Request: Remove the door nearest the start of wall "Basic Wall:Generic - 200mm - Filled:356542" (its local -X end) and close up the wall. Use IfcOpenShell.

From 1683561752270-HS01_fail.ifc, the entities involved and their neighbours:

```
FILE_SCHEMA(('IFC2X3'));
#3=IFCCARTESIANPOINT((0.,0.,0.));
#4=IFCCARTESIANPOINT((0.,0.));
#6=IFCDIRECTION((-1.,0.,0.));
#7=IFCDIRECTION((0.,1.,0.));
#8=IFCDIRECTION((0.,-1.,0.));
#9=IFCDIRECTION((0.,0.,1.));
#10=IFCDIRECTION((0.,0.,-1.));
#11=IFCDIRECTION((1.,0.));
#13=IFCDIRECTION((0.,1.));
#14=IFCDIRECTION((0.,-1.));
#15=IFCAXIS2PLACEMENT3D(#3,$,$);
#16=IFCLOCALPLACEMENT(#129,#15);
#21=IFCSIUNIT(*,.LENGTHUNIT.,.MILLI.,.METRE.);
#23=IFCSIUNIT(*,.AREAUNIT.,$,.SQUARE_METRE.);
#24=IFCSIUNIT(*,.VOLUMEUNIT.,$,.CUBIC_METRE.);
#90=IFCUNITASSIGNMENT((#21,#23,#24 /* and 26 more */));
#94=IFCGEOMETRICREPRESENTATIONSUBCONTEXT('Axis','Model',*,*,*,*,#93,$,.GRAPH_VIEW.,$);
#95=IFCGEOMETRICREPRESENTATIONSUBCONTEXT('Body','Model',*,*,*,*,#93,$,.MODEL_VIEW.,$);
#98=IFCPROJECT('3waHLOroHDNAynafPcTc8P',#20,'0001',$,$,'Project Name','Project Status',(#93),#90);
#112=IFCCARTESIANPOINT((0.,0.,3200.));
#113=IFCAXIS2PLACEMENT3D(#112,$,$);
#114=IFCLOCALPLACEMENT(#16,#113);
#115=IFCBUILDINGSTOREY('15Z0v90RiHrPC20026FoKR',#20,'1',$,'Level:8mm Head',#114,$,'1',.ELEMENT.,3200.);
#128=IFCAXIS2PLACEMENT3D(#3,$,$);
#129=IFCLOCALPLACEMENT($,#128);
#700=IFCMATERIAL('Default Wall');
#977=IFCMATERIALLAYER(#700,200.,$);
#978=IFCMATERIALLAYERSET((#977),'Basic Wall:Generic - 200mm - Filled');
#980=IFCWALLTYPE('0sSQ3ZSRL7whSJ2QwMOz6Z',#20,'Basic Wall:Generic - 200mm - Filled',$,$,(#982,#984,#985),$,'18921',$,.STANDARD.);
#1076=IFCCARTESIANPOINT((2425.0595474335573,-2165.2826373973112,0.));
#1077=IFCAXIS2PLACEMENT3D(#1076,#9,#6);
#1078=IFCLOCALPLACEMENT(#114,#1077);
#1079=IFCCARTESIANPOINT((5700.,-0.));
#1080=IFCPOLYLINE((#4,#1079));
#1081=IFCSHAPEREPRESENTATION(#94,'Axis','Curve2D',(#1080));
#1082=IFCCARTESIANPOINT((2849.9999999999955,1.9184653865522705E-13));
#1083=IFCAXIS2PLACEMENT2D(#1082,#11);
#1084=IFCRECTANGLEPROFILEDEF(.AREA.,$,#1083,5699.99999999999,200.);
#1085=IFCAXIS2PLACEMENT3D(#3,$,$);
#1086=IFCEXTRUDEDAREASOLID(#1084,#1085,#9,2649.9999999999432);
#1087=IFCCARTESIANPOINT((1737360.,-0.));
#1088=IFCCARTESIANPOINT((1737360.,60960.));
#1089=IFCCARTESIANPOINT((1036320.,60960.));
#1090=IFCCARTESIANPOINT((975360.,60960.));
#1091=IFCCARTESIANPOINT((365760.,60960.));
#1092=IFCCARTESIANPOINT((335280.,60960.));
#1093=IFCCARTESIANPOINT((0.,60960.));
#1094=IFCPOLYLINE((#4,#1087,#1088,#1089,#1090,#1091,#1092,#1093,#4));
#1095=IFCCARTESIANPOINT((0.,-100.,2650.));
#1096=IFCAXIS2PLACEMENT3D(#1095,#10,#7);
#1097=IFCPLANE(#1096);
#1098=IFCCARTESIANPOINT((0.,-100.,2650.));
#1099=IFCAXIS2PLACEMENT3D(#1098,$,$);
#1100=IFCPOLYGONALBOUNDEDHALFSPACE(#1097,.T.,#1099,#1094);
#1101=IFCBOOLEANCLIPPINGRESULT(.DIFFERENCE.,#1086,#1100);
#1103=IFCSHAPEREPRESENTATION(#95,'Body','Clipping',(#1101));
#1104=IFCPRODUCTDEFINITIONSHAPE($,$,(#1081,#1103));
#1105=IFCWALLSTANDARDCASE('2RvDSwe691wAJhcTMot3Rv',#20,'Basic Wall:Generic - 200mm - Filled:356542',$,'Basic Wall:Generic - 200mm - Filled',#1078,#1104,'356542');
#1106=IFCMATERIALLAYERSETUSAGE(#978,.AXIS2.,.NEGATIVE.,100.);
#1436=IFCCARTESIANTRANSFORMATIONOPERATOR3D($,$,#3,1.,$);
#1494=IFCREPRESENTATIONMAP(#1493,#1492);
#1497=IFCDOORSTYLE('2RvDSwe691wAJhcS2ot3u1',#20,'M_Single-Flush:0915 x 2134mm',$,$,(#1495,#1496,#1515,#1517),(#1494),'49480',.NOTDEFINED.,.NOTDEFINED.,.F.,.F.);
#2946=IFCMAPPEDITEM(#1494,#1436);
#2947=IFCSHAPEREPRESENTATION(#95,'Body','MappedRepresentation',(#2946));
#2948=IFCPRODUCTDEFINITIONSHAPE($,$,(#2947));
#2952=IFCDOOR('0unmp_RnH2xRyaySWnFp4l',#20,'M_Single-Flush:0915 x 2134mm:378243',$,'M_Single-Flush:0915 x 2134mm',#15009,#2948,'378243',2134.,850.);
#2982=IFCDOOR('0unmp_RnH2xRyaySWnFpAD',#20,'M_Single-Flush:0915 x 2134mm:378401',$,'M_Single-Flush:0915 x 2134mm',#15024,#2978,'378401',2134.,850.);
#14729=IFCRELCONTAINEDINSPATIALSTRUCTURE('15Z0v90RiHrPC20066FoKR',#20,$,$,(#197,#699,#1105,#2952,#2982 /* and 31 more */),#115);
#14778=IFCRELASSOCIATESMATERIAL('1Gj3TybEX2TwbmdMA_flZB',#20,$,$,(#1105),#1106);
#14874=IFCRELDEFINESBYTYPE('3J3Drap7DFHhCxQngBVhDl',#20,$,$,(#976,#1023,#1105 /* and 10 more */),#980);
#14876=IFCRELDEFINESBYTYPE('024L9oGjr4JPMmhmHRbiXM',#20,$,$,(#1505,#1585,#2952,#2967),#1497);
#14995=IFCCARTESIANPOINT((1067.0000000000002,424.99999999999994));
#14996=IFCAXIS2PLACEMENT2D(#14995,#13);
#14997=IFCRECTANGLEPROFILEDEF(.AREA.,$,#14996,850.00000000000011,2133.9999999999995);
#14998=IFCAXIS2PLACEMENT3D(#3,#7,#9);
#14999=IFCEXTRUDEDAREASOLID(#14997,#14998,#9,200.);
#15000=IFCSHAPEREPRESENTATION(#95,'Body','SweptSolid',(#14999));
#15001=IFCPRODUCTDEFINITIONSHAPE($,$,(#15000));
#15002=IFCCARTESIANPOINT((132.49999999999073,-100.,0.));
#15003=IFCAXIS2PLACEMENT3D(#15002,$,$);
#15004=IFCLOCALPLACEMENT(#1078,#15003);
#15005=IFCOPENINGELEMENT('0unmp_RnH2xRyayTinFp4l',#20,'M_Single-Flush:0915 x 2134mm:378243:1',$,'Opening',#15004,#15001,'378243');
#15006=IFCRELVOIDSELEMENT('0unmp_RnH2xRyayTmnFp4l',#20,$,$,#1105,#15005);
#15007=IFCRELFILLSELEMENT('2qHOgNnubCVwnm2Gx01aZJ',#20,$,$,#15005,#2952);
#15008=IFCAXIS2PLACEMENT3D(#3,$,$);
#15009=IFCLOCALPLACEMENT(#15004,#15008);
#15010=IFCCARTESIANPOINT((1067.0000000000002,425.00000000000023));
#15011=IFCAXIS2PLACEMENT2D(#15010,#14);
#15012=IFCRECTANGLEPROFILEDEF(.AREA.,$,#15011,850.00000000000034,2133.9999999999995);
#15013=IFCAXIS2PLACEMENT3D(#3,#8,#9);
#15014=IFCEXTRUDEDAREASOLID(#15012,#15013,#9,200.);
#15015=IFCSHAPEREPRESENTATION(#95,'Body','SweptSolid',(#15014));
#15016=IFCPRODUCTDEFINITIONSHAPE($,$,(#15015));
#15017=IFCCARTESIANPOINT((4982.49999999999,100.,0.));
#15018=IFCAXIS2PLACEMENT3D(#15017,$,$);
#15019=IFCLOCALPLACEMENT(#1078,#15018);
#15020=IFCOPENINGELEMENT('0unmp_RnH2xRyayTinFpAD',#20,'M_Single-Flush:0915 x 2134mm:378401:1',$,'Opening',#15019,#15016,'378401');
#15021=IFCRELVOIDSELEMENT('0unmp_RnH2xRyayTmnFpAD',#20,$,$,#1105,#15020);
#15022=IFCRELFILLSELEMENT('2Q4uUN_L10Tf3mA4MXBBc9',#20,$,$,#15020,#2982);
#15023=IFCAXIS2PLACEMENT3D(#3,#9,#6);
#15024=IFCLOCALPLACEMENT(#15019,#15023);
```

```python
import ifcopenshell
import ifcopenshell.api.feature
import ifcopenshell.api.root
import ifcopenshell.geom
import ifcopenshell.util.shape

model = ifcopenshell.open("1683561752270-HS01_fail.ifc")
settings = ifcopenshell.geom.settings()


def volume(element):
    """Net volume in cubic metres, openings subtracted."""
    shape = ifcopenshell.geom.create_shape(settings, element)
    return ifcopenshell.util.shape.get_volume(shape.geometry)


door = model.by_id(2952)
opening = door.FillsVoids[0].RelatingOpeningElement
wall = opening.VoidsElements[0].RelatingBuildingElement
before = volume(wall)

ifcopenshell.api.root.remove_product(model, product=door)
ifcopenshell.api.feature.remove_feature(model, feature=opening)

after = volume(wall)

print(f"wall volume {before:.3f} -> {after:.3f} m3")

model.write("1683561752270-HS01_fail_updated.ifc")
```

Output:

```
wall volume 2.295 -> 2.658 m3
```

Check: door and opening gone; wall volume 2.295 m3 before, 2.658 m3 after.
